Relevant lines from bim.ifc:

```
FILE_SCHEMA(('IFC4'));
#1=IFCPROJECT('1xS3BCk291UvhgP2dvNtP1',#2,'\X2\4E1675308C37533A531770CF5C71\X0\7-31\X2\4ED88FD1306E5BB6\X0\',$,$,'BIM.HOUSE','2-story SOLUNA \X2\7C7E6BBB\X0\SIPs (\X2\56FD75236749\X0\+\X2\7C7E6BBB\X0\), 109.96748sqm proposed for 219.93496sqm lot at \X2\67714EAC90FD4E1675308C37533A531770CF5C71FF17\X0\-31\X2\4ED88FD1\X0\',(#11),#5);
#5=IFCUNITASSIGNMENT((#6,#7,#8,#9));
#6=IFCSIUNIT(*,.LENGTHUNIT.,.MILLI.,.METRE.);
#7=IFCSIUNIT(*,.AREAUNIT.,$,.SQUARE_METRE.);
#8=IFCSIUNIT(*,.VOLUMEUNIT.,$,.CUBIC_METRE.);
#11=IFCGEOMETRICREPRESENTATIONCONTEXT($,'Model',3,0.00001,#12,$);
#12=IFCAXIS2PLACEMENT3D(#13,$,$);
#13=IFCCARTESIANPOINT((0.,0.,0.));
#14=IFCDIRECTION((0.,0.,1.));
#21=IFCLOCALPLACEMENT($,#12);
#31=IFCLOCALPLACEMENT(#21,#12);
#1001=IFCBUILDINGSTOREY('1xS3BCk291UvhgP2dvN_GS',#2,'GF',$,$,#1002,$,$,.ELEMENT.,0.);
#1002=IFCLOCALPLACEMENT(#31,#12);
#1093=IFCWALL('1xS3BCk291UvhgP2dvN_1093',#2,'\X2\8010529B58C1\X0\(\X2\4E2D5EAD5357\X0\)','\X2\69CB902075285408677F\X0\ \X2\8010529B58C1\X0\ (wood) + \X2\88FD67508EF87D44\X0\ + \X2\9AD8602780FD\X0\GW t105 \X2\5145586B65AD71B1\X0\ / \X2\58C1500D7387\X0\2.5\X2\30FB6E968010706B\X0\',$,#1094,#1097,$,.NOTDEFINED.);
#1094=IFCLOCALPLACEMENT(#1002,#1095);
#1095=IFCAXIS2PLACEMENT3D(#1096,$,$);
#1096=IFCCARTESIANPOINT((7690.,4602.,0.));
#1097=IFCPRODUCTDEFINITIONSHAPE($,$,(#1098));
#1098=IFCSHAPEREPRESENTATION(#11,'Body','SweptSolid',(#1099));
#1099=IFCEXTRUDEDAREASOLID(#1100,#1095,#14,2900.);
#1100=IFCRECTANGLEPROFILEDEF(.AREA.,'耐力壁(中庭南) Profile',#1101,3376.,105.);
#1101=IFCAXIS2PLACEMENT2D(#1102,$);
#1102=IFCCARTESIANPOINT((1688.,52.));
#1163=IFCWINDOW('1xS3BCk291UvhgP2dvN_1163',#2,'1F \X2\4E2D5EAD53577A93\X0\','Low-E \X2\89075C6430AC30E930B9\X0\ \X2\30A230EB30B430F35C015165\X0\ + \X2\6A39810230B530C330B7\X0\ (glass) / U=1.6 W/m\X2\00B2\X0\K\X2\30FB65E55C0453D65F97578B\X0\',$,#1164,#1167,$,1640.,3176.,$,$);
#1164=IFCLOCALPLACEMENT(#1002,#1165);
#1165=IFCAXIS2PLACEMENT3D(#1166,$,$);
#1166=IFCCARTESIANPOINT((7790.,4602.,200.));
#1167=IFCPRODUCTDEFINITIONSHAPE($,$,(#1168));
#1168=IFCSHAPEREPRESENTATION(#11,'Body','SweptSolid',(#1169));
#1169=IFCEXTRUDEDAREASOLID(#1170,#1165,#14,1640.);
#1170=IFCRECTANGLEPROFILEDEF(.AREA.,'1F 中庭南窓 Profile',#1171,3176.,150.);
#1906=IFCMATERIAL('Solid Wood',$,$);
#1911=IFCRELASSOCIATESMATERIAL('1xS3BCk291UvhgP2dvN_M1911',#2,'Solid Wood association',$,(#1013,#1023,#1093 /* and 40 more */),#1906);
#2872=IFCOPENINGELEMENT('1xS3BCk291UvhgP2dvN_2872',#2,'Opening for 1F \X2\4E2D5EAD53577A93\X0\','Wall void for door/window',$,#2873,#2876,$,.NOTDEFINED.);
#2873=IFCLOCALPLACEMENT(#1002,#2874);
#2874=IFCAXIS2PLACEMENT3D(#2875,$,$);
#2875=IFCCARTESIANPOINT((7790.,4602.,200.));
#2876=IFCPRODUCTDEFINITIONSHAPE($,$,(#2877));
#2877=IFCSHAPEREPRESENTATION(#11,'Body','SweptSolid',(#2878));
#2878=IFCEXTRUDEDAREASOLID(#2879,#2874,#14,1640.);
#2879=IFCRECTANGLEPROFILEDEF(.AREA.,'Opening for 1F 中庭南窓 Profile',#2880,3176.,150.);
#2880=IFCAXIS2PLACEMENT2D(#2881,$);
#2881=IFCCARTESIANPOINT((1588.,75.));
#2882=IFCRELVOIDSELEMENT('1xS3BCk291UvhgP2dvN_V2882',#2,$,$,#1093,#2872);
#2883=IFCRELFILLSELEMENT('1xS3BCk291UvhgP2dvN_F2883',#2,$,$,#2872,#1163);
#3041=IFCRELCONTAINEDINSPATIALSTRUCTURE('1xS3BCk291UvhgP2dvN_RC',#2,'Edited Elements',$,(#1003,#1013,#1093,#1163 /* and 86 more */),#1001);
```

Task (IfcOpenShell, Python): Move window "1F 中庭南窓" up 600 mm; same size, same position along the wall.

```python
import numpy as np
import ifcopenshell
import ifcopenshell.api.geometry
import ifcopenshell.util.placement
import ifcopenshell.util.unit

model = ifcopenshell.open("bim.ifc")
unit_scale = ifcopenshell.util.unit.calculate_unit_scale(model)

window = model.by_id(1163)
opening = window.FillsVoids[0].RelatingOpeningElement
dz = 600.0

shift = np.array([0.0, 0.0, dz])
# The window is not placed relative to its opening, so move both.
for product in (opening, window):
    matrix = ifcopenshell.util.placement.get_local_placement(product.ObjectPlacement)
    matrix[:3, 3] += shift
    ifcopenshell.api.geometry.edit_object_placement(model, product=product, matrix=matrix, is_si=False)

print(f"moved by {dz * unit_scale:+.3f} m")

model.write("bim-out.ifc")
```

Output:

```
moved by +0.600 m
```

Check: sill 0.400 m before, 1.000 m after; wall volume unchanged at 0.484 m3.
